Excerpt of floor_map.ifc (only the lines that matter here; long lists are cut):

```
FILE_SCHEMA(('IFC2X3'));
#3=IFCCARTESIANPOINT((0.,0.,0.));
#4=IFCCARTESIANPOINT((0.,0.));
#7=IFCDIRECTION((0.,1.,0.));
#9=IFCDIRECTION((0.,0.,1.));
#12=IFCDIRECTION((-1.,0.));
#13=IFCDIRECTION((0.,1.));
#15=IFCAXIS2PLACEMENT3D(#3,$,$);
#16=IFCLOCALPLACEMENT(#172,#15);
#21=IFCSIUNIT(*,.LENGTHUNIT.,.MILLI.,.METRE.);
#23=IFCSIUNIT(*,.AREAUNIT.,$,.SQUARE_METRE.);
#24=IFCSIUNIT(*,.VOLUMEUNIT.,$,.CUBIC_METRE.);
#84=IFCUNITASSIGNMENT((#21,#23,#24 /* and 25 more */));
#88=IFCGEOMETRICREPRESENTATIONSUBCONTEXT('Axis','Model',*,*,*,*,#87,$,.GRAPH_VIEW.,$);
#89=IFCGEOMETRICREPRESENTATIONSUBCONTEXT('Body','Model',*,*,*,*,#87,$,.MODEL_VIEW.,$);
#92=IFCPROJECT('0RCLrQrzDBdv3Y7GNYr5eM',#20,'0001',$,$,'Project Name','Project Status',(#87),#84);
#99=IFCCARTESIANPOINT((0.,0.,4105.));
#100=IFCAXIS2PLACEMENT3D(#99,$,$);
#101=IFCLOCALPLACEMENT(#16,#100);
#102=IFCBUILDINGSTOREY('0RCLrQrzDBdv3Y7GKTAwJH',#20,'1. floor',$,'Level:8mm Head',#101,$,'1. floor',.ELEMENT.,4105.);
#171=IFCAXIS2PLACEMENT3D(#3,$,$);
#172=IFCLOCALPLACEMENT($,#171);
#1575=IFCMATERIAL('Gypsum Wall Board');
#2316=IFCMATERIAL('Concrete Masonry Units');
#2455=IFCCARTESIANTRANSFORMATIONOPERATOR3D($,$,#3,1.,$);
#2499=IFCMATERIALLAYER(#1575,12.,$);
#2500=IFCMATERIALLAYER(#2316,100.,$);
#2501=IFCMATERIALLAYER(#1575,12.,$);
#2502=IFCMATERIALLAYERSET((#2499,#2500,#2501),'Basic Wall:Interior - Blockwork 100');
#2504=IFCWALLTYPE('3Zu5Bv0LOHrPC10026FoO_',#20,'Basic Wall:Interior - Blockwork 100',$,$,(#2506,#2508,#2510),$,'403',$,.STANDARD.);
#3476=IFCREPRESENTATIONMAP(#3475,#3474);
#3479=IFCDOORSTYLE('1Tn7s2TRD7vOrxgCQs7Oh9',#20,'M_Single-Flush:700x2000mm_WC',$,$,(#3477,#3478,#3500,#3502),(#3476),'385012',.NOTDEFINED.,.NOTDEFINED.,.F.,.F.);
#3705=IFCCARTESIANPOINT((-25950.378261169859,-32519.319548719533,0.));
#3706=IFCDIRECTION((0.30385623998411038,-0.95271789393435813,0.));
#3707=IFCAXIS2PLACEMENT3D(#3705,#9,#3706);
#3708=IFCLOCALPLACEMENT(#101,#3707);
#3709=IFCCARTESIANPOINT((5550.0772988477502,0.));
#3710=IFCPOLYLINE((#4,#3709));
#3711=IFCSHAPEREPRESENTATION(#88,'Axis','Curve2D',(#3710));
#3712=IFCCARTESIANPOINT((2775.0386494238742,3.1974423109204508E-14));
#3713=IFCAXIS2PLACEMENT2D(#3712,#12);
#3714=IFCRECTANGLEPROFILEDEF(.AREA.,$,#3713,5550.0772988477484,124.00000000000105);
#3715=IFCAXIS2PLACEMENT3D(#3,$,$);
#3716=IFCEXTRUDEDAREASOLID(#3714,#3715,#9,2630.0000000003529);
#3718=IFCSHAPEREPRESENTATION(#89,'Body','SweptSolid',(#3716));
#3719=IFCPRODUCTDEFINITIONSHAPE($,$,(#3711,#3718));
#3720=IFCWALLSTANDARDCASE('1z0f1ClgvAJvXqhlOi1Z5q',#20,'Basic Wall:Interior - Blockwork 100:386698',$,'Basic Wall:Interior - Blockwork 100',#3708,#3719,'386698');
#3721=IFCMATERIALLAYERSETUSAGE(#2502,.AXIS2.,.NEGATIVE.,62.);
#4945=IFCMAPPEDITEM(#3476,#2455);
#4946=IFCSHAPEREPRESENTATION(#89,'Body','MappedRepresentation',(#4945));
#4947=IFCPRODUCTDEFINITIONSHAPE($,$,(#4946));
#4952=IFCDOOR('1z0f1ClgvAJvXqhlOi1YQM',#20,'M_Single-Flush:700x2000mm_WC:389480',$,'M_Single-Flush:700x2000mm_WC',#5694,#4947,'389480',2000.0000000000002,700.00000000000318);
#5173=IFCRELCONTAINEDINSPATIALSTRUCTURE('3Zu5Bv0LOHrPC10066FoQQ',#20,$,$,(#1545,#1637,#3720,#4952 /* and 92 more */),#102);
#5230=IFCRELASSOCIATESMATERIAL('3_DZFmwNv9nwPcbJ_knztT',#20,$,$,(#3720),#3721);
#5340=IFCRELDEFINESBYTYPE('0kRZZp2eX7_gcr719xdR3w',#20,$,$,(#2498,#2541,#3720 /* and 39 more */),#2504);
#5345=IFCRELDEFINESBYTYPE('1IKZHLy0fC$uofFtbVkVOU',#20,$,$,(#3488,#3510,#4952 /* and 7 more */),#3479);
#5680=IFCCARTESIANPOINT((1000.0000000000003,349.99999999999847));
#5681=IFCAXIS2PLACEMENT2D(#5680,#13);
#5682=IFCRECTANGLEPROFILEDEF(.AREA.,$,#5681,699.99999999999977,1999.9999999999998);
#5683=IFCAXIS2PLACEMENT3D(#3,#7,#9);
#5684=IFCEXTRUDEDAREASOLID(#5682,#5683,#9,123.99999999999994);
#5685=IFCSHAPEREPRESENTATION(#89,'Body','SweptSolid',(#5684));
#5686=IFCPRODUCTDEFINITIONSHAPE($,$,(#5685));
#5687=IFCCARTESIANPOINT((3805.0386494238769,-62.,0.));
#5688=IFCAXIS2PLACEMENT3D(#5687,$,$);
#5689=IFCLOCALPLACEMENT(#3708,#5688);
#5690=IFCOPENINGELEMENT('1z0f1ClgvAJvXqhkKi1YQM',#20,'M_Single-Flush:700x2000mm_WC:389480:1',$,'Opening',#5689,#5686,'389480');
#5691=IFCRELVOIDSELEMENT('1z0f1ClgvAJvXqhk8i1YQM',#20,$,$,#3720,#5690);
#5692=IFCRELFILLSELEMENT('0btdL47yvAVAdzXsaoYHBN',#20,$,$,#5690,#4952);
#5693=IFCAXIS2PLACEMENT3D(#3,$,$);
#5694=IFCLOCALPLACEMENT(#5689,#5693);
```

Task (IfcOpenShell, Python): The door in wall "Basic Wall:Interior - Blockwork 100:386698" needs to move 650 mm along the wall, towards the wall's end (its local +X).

```python
import ifcopenshell
import ifcopenshell.api.geometry
import ifcopenshell.util.placement
import ifcopenshell.util.unit

model = ifcopenshell.open("floor_map.ifc")
unit_scale = ifcopenshell.util.unit.calculate_unit_scale(model)

door = model.by_id(4952)
opening = door.FillsVoids[0].RelatingOpeningElement
wall = opening.VoidsElements[0].RelatingBuildingElement

wall_matrix = ifcopenshell.util.placement.get_local_placement(wall.ObjectPlacement)
shift = wall_matrix[:3, 0] * 0.65 / unit_scale
before = ifcopenshell.util.placement.get_local_placement(door.ObjectPlacement)[:3, 3].copy()

# The door is placed relative to its opening, so it follows when the opening moves.
matrix = ifcopenshell.util.placement.get_local_placement(opening.ObjectPlacement)
matrix[:3, 3] += shift
ifcopenshell.api.geometry.edit_object_placement(
    model, product=opening, matrix=matrix, is_si=False, should_transform_children=True
)

after = ifcopenshell.util.placement.get_local_placement(door.ObjectPlacement)[:3, 3]
print("door moved by", (after - before).round(3) + 0.0)

model.write("floor_map_v2.ifc")
```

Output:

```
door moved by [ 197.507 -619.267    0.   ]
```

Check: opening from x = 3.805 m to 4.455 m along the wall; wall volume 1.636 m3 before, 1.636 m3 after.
